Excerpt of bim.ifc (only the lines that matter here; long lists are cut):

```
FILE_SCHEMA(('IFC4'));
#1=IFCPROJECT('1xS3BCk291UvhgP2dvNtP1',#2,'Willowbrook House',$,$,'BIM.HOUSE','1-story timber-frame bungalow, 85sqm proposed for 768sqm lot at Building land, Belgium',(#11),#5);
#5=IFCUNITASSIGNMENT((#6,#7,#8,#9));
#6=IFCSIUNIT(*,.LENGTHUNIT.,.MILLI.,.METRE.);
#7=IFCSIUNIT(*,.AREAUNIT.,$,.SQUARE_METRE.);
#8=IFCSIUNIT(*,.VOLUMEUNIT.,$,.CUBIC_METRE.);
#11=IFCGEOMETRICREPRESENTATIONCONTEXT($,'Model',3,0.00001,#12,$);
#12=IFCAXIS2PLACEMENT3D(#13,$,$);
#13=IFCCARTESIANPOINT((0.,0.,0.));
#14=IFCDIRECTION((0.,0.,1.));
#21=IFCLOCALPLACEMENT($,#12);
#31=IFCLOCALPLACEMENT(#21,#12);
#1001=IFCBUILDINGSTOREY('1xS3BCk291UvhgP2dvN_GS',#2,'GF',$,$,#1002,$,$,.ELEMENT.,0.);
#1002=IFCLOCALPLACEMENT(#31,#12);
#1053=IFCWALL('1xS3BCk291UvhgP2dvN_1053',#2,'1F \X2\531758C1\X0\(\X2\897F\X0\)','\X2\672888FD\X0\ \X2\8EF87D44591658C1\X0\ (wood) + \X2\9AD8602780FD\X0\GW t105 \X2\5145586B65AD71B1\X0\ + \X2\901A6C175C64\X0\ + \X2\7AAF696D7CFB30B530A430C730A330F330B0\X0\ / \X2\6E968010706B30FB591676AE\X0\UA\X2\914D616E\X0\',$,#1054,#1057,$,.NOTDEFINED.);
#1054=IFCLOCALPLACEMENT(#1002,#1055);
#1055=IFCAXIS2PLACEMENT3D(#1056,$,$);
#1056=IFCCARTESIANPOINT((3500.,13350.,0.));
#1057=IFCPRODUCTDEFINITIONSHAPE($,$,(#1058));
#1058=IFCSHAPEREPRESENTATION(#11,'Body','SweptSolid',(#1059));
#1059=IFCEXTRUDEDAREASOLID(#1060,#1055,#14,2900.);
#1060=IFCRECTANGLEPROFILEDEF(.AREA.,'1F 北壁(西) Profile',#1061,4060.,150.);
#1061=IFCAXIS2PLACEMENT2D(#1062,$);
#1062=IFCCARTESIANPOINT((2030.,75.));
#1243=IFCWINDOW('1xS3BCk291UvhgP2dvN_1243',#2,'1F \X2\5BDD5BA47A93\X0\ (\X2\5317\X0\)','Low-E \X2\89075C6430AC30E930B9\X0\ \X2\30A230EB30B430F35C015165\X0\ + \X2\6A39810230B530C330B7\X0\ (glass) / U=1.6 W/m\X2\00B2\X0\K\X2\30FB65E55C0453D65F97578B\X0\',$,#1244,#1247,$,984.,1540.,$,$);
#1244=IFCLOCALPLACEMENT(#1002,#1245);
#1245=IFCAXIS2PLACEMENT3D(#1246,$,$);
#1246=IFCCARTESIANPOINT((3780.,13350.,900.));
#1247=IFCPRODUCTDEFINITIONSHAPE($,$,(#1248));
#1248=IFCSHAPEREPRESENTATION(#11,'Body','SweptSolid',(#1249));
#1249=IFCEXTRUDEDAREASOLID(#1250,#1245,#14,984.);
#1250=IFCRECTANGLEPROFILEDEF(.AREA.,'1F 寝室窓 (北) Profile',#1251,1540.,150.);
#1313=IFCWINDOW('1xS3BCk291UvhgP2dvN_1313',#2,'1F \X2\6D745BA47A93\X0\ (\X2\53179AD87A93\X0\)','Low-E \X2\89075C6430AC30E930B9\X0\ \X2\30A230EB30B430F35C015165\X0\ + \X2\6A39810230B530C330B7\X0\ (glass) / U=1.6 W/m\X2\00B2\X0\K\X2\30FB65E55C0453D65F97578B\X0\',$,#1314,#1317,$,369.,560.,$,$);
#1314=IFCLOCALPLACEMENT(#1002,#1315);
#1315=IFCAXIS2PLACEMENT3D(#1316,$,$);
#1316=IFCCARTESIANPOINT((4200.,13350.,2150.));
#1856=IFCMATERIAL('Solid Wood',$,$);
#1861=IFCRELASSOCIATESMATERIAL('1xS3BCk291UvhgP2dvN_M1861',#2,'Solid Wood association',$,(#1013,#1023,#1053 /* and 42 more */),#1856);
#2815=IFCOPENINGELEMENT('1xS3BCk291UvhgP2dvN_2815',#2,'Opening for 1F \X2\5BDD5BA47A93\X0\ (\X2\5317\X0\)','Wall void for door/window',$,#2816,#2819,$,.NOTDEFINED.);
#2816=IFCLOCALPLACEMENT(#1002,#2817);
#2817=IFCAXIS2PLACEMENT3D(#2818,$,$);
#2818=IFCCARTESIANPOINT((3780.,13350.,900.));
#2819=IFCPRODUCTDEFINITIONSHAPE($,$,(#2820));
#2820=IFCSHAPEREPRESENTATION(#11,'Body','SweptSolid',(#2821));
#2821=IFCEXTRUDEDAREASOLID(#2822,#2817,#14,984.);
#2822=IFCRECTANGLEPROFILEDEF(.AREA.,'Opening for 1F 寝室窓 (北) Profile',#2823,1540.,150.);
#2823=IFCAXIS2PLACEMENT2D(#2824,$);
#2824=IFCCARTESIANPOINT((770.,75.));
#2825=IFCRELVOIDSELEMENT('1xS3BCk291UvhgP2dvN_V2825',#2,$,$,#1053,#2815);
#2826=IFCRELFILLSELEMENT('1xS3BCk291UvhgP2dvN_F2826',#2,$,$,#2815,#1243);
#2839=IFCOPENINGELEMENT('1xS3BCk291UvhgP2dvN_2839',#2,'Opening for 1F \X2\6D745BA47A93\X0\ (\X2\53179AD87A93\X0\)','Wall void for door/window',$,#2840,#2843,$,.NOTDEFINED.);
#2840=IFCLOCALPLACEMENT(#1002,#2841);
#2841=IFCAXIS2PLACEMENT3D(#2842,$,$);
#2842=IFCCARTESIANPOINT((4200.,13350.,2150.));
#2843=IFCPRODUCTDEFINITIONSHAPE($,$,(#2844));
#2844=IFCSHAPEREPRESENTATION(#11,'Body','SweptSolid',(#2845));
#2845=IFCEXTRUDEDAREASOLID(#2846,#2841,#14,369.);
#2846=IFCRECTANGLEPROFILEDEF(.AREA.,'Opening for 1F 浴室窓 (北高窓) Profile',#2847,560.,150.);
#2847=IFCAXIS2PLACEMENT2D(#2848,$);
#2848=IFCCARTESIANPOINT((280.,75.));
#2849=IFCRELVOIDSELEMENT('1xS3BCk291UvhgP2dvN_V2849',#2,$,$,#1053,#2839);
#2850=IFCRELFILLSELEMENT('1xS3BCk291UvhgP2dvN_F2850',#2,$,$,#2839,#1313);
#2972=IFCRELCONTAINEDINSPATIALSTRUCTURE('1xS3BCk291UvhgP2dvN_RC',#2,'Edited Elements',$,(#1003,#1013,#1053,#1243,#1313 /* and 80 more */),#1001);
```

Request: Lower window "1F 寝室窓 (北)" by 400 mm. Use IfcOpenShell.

```python
import numpy as np
import ifcopenshell
import ifcopenshell.api.geometry
import ifcopenshell.util.placement
import ifcopenshell.util.unit

model = ifcopenshell.open("bim.ifc")
unit_scale = ifcopenshell.util.unit.calculate_unit_scale(model)

window = model.by_id(1243)
opening = window.FillsVoids[0].RelatingOpeningElement
dz = -0.4 / unit_scale

shift = np.array([0.0, 0.0, dz])
# The window is not placed relative to its opening, so move both.
for product in (opening, window):
    matrix = ifcopenshell.util.placement.get_local_placement(product.ObjectPlacement)
    matrix[:3, 3] += shift
    ifcopenshell.api.geometry.edit_object_placement(model, product=product, matrix=matrix, is_si=False)

print(f"moved by {dz * unit_scale:+.3f} m")

model.write("bim_updated.ifc")
```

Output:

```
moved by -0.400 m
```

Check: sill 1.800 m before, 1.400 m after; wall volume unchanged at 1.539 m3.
